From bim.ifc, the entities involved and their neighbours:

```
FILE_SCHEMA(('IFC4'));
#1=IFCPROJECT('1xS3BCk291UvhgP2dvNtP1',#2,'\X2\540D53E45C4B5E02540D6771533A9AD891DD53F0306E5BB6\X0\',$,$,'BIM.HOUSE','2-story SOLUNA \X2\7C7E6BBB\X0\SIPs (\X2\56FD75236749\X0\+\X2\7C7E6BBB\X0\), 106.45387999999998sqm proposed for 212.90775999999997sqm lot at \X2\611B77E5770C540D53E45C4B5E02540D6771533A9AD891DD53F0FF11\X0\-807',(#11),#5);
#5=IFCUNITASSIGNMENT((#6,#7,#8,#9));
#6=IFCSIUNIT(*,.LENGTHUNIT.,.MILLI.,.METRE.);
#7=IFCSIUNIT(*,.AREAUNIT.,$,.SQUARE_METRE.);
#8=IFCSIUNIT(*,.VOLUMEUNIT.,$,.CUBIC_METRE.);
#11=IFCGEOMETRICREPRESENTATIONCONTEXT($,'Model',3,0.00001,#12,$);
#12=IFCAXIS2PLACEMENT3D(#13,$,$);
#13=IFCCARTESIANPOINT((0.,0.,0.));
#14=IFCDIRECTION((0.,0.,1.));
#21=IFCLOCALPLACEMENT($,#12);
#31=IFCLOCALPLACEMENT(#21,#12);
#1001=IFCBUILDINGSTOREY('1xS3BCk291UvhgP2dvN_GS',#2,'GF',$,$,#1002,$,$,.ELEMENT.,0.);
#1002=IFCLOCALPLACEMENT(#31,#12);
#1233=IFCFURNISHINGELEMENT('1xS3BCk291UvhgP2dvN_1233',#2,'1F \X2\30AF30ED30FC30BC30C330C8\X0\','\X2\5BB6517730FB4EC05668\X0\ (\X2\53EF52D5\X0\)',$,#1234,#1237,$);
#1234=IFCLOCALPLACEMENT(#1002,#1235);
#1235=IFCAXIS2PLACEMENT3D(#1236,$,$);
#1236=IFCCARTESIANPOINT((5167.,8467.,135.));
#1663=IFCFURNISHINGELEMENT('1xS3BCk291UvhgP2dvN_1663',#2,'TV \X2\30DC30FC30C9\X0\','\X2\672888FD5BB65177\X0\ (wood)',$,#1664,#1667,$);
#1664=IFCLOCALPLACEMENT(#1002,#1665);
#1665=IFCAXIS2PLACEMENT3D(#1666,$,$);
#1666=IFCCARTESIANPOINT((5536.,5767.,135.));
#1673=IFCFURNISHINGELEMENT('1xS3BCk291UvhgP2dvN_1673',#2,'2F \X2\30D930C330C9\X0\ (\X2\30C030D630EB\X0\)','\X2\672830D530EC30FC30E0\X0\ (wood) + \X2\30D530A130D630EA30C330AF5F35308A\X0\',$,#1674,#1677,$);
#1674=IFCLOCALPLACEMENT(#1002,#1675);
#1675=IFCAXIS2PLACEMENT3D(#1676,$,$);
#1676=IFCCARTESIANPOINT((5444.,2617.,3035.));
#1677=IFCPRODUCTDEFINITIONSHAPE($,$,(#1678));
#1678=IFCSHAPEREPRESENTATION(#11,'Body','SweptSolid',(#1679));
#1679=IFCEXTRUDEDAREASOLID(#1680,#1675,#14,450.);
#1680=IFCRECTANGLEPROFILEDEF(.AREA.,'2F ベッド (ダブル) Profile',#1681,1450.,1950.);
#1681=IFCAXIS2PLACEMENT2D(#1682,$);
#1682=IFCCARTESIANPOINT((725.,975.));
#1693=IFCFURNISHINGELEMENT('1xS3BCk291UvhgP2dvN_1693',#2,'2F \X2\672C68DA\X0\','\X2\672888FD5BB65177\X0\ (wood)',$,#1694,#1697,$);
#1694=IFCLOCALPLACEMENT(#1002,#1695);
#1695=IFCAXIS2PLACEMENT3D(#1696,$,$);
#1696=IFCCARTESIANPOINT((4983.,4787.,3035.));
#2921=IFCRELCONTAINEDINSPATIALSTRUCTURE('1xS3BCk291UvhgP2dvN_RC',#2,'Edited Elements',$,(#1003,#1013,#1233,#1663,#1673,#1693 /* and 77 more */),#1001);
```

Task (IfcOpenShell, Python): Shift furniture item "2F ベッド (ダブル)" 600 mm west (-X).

```python
import ifcopenshell
import ifcopenshell.api.geometry
import ifcopenshell.util.placement
import ifcopenshell.util.unit

model = ifcopenshell.open("bim.ifc")
unit_scale = ifcopenshell.util.unit.calculate_unit_scale(model)

item = model.by_guid("1xS3BCk291UvhgP2dvN_1673")
matrix = ifcopenshell.util.placement.get_local_placement(item.ObjectPlacement)
matrix[0, 3] -= 0.6 / unit_scale
ifcopenshell.api.geometry.edit_object_placement(model, product=item, matrix=matrix, is_si=False)

print(ifcopenshell.util.placement.get_local_placement(item.ObjectPlacement).round(3) + 0.0)

model.write("bim_v2.ifc")
```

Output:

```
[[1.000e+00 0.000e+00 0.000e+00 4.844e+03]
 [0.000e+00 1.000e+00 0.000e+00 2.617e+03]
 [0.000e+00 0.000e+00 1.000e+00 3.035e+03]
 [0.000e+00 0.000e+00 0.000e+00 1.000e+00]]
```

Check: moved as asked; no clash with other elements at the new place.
